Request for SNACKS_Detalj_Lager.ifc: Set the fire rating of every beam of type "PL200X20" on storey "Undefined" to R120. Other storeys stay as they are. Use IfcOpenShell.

First a look at what the model holds.

```python
import ifcopenshell
import ifcopenshell.util.element

model = ifcopenshell.open("SNACKS_Detalj_Lager.ifc")
print(model.schema)
storey = next(s for s in model.by_type("IfcBuildingStorey") if s.Name == "Undefined")
beams = [e for e in ifcopenshell.util.element.get_decomposition(storey) if e.is_a("IfcBeam")]
seen = {}
for e in beams:
    element_type = ifcopenshell.util.element.get_type(e)
    key = (element_type.Name if element_type != e and element_type else None, ifcopenshell.util.element.get_pset(e, "Pset_BeamCommon", "FireRating"))
    seen[key] = seen.get(key, 0) + 1
for (name, value), count in sorted(seen.items(), key=str):
    print(count, "x", name, "|", value)
```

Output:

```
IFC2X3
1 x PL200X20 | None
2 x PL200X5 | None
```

```python
import ifcopenshell
import ifcopenshell.api.pset
import ifcopenshell.util.element

model = ifcopenshell.open("SNACKS_Detalj_Lager.ifc")

storey = next(s for s in model.by_type("IfcBuildingStorey") if s.Name == "Undefined")
beams = [e for e in ifcopenshell.util.element.get_decomposition(storey) if e.is_a("IfcBeam")]

count = 0
for e in beams:
    element_type = ifcopenshell.util.element.get_type(e)
    if element_type in (None, e) or element_type.Name != "PL200X20":
        continue
    # add_pset returns the element's existing set when there is one.
    pset = ifcopenshell.api.pset.add_pset(model, product=e, name="Pset_BeamCommon")
    ifcopenshell.api.pset.edit_pset(model, pset=pset, properties={"FireRating": "R120"})
    count += 1

print(count, "beams updated")

model.write("SNACKS_Detalj_Lager_rev.ifc")
```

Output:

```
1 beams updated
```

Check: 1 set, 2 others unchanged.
